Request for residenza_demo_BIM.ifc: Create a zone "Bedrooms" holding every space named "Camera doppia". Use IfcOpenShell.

First a look at what the model holds.

```python
import ifcopenshell

model = ifcopenshell.open("residenza_demo_BIM.ifc")
print(model.schema)
seen = {}
for space in model.by_type("IfcSpace"):
    seen[space.LongName] = seen.get(space.LongName, 0) + 1
for name, count in sorted(seen.items(), key=str):
    print(count, "x", name)
print("zones:", [z.Name for z in model.by_type("IfcZone")][:20])
```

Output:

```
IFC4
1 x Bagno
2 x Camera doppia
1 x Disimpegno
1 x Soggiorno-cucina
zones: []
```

```python
import ifcopenshell
import ifcopenshell.api.group
import ifcopenshell.api.root

model = ifcopenshell.open("residenza_demo_BIM.ifc")

names = {"Camera doppia"}
spaces = [s for s in model.by_type("IfcSpace") if s.LongName in names]

zone = ifcopenshell.api.root.create_entity(model, ifc_class="IfcZone", name="Bedrooms")
ifcopenshell.api.group.assign_group(model, products=spaces, group=zone)
print(len(spaces), "spaces in", zone.Name)

model.write("residenza_demo_BIM_edited.ifc")
```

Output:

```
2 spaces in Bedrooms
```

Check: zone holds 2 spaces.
